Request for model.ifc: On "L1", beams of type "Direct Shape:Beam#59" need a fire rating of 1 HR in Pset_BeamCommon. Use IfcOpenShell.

First a look at what the model holds.

```python
import ifcopenshell
import ifcopenshell.util.element

model = ifcopenshell.open("model.ifc")
print(model.schema)
storey = next(s for s in model.by_type("IfcBuildingStorey") if s.Name == "L1")
beams = [e for e in ifcopenshell.util.element.get_decomposition(storey) if e.is_a("IfcBeam")]
seen = {}
for e in beams:
    element_type = ifcopenshell.util.element.get_type(e)
    key = (element_type.Name if element_type != e and element_type else None, ifcopenshell.util.element.get_pset(e, "Pset_BeamCommon", "FireRating"))
    seen[key] = seen.get(key, 0) + 1
for (name, value), count in sorted(seen.items(), key=str):
    print(count, "x", name, "|", value)
```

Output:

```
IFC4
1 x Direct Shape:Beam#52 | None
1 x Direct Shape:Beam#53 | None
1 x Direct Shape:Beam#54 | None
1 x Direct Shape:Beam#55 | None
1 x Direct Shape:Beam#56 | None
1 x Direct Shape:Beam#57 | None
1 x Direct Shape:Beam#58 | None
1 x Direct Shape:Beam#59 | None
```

```python
import ifcopenshell
import ifcopenshell.api.pset
import ifcopenshell.util.element

model = ifcopenshell.open("model.ifc")

storey = next(s for s in model.by_type("IfcBuildingStorey") if s.Name == "L1")
beams = [e for e in ifcopenshell.util.element.get_decomposition(storey) if e.is_a("IfcBeam")]

count = 0
for e in beams:
    element_type = ifcopenshell.util.element.get_type(e)
    if element_type in (None, e) or element_type.Name != "Direct Shape:Beam#59":
        continue
    # add_pset returns the element's existing set when there is one.
    pset = ifcopenshell.api.pset.add_pset(model, product=e, name="Pset_BeamCommon")
    ifcopenshell.api.pset.edit_pset(model, pset=pset, properties={"FireRating": "1 HR"})
    count += 1

print(count, "beams updated")

model.write("model_v2.ifc")
```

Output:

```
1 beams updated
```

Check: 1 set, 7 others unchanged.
